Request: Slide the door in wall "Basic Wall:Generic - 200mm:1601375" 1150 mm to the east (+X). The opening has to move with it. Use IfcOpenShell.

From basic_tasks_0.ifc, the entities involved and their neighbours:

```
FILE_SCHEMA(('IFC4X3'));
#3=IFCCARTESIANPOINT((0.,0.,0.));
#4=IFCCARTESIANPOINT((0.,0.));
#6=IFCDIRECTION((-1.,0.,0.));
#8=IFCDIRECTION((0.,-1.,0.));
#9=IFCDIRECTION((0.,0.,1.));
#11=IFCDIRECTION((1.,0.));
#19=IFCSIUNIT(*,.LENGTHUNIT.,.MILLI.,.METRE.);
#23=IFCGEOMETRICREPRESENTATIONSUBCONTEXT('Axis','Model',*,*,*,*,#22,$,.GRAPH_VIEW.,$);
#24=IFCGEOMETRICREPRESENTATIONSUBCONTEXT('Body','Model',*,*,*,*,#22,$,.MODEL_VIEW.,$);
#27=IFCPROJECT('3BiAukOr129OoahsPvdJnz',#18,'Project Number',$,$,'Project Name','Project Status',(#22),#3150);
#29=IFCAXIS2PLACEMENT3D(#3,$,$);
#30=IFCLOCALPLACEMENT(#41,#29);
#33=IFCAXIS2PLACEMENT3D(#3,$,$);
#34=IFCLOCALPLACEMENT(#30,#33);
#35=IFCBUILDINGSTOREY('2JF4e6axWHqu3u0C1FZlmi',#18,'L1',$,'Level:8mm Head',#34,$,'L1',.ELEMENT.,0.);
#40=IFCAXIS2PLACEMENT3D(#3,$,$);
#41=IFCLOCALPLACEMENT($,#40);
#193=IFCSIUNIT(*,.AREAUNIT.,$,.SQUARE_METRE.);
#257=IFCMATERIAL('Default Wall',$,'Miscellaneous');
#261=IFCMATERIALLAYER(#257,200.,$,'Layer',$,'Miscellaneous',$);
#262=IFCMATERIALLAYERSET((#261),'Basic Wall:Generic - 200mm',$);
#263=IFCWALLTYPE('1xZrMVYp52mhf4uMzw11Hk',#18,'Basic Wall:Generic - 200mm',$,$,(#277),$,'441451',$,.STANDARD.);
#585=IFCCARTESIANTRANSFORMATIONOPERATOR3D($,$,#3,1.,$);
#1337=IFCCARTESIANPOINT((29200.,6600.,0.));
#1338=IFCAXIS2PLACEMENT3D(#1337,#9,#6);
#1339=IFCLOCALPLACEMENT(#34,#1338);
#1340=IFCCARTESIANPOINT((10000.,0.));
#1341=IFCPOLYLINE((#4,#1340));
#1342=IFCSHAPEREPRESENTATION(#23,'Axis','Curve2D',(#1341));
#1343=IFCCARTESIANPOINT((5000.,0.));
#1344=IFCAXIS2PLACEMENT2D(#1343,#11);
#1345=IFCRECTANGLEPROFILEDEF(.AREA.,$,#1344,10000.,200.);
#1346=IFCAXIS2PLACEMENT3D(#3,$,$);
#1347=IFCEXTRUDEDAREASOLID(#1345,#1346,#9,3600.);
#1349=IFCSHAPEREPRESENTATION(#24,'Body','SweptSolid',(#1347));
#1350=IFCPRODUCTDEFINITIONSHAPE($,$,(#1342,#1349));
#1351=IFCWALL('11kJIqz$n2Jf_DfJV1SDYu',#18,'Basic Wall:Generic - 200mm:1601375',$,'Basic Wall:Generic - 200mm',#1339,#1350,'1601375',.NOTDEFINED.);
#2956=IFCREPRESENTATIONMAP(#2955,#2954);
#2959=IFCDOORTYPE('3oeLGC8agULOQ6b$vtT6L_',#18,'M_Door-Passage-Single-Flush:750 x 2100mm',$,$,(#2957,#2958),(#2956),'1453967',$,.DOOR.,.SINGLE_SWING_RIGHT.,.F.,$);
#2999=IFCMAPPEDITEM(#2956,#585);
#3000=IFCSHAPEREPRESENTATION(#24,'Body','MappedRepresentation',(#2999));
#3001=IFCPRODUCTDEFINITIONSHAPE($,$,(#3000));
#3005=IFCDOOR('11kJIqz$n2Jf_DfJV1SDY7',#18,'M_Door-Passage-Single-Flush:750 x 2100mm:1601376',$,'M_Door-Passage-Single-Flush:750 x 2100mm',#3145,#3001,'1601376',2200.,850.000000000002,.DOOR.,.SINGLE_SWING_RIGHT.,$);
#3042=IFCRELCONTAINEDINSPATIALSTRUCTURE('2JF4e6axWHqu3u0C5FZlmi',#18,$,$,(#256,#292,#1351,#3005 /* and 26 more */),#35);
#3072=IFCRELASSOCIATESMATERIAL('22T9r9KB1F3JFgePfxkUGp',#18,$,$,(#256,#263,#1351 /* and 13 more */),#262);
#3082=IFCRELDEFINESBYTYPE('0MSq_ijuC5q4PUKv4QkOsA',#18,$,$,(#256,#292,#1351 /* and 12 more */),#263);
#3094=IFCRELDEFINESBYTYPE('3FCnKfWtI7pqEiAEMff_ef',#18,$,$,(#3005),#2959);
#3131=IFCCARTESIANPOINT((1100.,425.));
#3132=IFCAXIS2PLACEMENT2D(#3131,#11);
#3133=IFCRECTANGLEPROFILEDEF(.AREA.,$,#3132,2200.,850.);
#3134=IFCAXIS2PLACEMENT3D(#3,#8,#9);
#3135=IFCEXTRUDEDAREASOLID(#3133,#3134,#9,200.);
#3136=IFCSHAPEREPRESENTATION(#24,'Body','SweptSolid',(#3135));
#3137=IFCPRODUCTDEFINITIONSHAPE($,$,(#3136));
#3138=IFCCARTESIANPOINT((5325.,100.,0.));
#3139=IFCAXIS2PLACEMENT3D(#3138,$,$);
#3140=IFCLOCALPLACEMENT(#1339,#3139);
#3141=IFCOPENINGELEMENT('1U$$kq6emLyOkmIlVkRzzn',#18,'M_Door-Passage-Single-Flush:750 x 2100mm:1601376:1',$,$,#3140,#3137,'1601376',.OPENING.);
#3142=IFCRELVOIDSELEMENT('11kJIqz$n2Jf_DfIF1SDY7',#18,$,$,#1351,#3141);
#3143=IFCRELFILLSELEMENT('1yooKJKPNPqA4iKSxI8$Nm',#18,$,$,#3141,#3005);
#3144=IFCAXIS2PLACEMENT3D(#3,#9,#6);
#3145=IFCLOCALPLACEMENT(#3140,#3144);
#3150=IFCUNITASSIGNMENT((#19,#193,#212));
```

```python
import ifcopenshell
import ifcopenshell.api.geometry
import ifcopenshell.util.placement

model = ifcopenshell.open("basic_tasks_0.ifc")

door = model.by_id(3005)
opening = door.FillsVoids[0].RelatingOpeningElement
wall = opening.VoidsElements[0].RelatingBuildingElement

wall_matrix = ifcopenshell.util.placement.get_local_placement(wall.ObjectPlacement)
shift = wall_matrix[:3, 0] * -1150.0
before = ifcopenshell.util.placement.get_local_placement(door.ObjectPlacement)[:3, 3].copy()

# The door is placed relative to its opening, so it follows when the opening moves.
matrix = ifcopenshell.util.placement.get_local_placement(opening.ObjectPlacement)
matrix[:3, 3] += shift
ifcopenshell.api.geometry.edit_object_placement(
    model, product=opening, matrix=matrix, is_si=False, should_transform_children=True
)

after = ifcopenshell.util.placement.get_local_placement(door.ObjectPlacement)[:3, 3]
print("door moved by", (after - before).round(3) + 0.0)

model.write("basic_tasks_0-out.ifc")
```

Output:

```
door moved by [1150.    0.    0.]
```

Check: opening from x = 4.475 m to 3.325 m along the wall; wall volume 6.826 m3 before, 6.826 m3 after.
